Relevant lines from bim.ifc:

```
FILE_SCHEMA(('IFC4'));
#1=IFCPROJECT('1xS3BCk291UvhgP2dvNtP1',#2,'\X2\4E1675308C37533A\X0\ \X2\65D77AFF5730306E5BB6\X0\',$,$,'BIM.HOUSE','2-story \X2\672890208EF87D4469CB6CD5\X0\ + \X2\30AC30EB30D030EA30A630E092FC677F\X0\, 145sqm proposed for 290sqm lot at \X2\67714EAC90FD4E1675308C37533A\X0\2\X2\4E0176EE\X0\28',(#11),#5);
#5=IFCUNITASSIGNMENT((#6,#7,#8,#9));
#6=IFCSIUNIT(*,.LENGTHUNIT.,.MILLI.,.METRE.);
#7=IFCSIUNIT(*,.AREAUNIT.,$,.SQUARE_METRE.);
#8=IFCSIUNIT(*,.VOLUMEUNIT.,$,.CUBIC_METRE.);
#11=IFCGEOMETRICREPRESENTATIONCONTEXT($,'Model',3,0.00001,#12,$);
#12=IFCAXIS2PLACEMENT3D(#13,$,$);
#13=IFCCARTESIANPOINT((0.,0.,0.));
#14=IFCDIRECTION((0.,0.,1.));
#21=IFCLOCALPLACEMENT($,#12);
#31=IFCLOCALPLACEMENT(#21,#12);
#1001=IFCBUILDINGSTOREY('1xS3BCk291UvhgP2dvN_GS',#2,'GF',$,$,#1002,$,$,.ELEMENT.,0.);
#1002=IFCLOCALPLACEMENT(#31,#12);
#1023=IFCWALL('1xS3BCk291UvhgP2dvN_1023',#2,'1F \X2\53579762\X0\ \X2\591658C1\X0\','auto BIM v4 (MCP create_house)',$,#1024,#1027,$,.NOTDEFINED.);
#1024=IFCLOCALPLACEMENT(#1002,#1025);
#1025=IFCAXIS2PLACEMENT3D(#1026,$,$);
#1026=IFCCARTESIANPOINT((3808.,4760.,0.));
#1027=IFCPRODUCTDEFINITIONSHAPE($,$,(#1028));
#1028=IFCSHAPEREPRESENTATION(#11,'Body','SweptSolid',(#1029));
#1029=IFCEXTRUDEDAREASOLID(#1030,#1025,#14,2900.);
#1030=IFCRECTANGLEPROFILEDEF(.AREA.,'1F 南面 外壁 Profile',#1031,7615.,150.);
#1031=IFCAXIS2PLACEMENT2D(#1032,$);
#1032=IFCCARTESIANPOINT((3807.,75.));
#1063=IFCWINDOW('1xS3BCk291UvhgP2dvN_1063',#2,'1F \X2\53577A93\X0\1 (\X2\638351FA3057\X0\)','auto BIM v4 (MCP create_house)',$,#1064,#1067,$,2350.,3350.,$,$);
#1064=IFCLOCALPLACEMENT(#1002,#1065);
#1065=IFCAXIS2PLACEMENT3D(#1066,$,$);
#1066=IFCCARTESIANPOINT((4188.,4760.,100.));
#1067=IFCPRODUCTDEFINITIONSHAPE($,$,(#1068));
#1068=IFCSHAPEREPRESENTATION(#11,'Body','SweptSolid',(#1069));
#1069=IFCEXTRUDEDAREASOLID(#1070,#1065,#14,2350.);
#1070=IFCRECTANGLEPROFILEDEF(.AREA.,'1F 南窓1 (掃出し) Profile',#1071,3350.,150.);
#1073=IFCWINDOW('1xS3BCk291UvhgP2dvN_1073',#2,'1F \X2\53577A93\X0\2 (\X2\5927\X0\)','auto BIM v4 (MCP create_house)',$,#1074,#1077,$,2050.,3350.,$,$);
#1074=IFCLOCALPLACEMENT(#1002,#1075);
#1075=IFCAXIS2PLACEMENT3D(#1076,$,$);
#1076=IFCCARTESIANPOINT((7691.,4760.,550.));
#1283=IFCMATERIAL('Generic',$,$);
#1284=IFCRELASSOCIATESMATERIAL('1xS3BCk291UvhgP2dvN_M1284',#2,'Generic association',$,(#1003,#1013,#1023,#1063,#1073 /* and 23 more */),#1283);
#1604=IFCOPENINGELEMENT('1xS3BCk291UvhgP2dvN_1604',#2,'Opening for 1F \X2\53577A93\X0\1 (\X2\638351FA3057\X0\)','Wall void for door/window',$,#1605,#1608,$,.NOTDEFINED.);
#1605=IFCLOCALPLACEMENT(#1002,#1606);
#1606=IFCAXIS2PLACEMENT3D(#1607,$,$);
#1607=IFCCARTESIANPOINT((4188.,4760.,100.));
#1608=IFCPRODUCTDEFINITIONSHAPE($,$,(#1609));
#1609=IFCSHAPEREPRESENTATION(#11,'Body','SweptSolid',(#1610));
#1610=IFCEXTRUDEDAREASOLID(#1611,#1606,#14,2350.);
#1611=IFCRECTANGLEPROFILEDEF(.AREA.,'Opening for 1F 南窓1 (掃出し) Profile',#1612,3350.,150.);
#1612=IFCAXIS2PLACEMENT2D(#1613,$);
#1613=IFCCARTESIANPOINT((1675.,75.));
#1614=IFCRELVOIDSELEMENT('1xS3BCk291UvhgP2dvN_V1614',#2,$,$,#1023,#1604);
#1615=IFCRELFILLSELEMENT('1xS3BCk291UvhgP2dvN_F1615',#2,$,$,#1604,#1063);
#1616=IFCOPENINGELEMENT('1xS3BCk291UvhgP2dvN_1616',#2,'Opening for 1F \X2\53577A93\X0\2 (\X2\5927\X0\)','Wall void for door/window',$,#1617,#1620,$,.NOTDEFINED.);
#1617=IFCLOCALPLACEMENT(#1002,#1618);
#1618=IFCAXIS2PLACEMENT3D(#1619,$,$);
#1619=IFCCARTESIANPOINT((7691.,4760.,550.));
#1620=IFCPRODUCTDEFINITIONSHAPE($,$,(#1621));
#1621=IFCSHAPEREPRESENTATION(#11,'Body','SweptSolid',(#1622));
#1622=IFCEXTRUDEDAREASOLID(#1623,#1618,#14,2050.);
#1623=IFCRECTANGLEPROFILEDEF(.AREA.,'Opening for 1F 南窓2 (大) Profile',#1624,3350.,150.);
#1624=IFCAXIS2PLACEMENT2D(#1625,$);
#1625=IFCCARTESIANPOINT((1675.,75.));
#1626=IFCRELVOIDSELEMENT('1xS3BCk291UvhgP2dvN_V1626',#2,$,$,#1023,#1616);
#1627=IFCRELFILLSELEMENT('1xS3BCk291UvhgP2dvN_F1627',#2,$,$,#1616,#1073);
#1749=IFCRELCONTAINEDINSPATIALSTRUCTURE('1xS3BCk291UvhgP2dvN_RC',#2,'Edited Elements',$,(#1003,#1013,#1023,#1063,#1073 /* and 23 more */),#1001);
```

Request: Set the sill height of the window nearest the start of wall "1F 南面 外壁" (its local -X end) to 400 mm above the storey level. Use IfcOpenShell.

```python
import numpy as np
import ifcopenshell
import ifcopenshell.api.geometry
import ifcopenshell.geom
import ifcopenshell.util.element
import ifcopenshell.util.placement
import ifcopenshell.util.shape
import ifcopenshell.util.unit

model = ifcopenshell.open("bim.ifc")
unit_scale = ifcopenshell.util.unit.calculate_unit_scale(model)

window = model.by_id(1063)
opening = window.FillsVoids[0].RelatingOpeningElement
storey = ifcopenshell.util.element.get_container(window, ifc_class="IfcBuildingStorey")
level = ifcopenshell.util.placement.get_local_placement(storey.ObjectPlacement)[2, 3]

# The opening's origin need not be at the sill, so measure its lowest point.
shape = ifcopenshell.geom.create_shape(ifcopenshell.geom.settings(), opening)
bottom = ifcopenshell.util.shape.get_shape_bottom_elevation(shape, shape.geometry) / unit_scale
dz = level + 400.0 - bottom

shift = np.array([0.0, 0.0, dz])
# The window is not placed relative to its opening, so move both.
for product in (opening, window):
    matrix = ifcopenshell.util.placement.get_local_placement(product.ObjectPlacement)
    matrix[:3, 3] += shift
    ifcopenshell.api.geometry.edit_object_placement(model, product=product, matrix=matrix, is_si=False)

print(f"moved by {dz * unit_scale:+.3f} m")

model.write("bim_v2.ifc")
```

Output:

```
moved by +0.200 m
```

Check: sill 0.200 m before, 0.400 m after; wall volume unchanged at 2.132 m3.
